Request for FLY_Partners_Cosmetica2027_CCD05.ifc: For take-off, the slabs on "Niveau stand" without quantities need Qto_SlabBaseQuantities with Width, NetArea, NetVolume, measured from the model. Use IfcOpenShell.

First a look at what the model holds.

```python
import ifcopenshell
import ifcopenshell.util.element
import ifcopenshell.util.unit

model = ifcopenshell.open("FLY_Partners_Cosmetica2027_CCD05.ifc")
print(model.schema)
for unit_type in ("LENGTHUNIT", "AREAUNIT", "VOLUMEUNIT"):
    print(unit_type, ifcopenshell.util.unit.calculate_unit_scale(model, unit_type))
storey = next(s for s in model.by_type("IfcBuildingStorey") if s.Name == "Niveau stand")
slabs = [e for e in ifcopenshell.util.element.get_decomposition(storey) if e.is_a("IfcSlab")]
for e in sorted(slabs, key=lambda e: e.id()):
    print(e.id(), e.is_a(), e.Name, list(ifcopenshell.util.element.get_psets(e, qtos_only=True)), sep=" | ")
```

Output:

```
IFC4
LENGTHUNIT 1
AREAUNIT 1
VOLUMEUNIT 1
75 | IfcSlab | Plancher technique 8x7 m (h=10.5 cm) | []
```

```python
import ifcopenshell
import ifcopenshell.api.pset
import ifcopenshell.geom
import ifcopenshell.util.element
import ifcopenshell.util.shape
import ifcopenshell.util.unit

model = ifcopenshell.open("FLY_Partners_Cosmetica2027_CCD05.ifc")
unit_scale = ifcopenshell.util.unit.calculate_unit_scale(model)
area_scale = ifcopenshell.util.unit.calculate_unit_scale(model, "AREAUNIT")
volume_scale = ifcopenshell.util.unit.calculate_unit_scale(model, "VOLUMEUNIT")
settings = ifcopenshell.geom.settings()

storey = next(s for s in model.by_type("IfcBuildingStorey") if s.Name == "Niveau stand")
slabs = [e for e in ifcopenshell.util.element.get_decomposition(storey) if e.is_a("IfcSlab")]

for e in sorted(slabs, key=lambda e: e.id()):
    if ifcopenshell.util.element.get_psets(e, qtos_only=True, should_inherit=False):
        continue
    # Geometry comes back in metres, in the element's own axes.
    shape = ifcopenshell.geom.create_shape(settings, e)
    values = {
        "Width": ifcopenshell.util.shape.get_z(shape.geometry) / unit_scale,
        "NetArea": ifcopenshell.util.shape.get_footprint_area(shape.geometry) / area_scale,
        "NetVolume": ifcopenshell.util.shape.get_volume(shape.geometry) / volume_scale,
    }
    qto = ifcopenshell.api.pset.add_qto(model, product=e, name="Qto_SlabBaseQuantities")
    ifcopenshell.api.pset.edit_qto(model, qto=qto, properties=values)
    print(e.id(), {k: round(v, 3) for k, v in values.items()})

model.write("FLY_Partners_Cosmetica2027_CCD05-out.ifc")
```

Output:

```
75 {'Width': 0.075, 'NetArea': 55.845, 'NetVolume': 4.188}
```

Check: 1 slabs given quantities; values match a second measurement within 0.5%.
